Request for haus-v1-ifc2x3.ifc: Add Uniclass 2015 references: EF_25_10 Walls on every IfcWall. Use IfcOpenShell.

First a look at what the model holds.

```python
import ifcopenshell

model = ifcopenshell.open("haus-v1-ifc2x3.ifc")
print(model.schema)
print("classifications:", [c.Name for c in model.by_type("IfcClassification")])
for ifc_class in ("IfcDoor", "IfcRoof", "IfcStair", "IfcWall", "IfcWindow"):
    print(ifc_class, len(model.by_type(ifc_class)))
```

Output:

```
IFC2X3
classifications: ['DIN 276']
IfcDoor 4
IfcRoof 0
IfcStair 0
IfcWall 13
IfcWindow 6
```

```python
import ifcopenshell
import ifcopenshell.api.classification

model = ifcopenshell.open("haus-v1-ifc2x3.ifc")

# IFC2X3 requires Source and Edition and has no link from the project to the system.
system = model.create_entity("IfcClassification", Source="NBS", Edition="2015", Name="Uniclass 2015")

codes = {
    "IfcWall": ("EF_25_10", "Walls"),
}
for ifc_class, (code, name) in codes.items():
    products = model.by_type(ifc_class)
    ifcopenshell.api.classification.add_reference(
        model, products=products, classification=system, identification=code, name=name
    )
    print(code, len(products))

model.write("haus-v1-ifc2x3-out.ifc")
```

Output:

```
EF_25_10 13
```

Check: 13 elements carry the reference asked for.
